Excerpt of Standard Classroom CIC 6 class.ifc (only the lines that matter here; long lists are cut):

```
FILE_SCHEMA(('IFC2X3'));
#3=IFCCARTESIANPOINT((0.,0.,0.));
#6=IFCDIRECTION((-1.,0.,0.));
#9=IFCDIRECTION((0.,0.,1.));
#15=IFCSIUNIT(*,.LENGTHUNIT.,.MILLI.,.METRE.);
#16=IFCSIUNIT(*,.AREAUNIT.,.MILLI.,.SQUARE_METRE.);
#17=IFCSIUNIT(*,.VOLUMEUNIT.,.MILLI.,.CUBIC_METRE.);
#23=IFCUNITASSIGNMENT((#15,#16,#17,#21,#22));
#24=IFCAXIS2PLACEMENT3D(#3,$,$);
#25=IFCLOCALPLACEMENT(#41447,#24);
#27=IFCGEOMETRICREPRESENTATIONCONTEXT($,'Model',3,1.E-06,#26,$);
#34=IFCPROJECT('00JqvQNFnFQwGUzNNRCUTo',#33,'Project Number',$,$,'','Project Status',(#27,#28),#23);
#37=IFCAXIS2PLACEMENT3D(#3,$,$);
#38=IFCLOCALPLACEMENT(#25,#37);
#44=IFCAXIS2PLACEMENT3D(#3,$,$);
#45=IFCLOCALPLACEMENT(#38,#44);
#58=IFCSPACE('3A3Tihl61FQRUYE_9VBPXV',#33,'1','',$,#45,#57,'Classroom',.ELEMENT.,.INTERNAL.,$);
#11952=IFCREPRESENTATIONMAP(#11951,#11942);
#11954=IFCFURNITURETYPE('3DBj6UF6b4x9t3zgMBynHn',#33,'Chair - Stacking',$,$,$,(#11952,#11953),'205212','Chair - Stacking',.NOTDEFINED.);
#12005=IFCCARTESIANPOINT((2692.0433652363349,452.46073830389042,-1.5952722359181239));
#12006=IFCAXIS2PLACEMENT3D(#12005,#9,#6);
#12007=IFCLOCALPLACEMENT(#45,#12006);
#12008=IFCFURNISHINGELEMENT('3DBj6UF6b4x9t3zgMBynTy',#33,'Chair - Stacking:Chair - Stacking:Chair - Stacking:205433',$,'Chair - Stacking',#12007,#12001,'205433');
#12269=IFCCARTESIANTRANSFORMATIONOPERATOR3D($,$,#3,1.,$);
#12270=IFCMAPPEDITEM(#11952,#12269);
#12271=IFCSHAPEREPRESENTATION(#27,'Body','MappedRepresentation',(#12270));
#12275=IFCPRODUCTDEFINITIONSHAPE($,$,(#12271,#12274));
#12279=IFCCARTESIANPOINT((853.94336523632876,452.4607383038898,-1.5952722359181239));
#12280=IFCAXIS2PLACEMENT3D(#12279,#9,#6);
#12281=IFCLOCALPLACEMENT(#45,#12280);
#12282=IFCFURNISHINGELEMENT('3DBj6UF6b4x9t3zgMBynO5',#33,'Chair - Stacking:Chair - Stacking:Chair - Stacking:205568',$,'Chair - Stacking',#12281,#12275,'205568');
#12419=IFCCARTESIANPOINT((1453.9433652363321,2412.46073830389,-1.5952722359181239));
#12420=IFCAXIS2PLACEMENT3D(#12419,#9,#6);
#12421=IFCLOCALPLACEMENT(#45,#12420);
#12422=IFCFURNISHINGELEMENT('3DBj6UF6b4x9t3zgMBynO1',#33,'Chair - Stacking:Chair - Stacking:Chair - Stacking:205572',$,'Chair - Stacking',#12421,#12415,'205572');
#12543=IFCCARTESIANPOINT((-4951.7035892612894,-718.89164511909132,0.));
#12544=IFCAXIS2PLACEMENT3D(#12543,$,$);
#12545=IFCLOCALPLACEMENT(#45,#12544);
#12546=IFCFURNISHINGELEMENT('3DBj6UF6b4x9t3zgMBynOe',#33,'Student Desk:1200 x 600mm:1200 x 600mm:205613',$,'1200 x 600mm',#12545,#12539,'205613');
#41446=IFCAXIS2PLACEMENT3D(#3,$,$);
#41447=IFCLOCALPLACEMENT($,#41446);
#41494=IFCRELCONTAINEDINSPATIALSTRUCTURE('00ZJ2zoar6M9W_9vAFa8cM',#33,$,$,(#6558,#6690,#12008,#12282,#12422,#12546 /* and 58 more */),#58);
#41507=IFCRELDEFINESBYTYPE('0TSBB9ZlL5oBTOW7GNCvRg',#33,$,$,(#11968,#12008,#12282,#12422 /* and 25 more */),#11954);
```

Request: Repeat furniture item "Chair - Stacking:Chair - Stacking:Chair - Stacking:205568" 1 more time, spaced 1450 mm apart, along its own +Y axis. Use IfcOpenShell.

```python
import ifcopenshell
import ifcopenshell.api.geometry
import ifcopenshell.api.root
import ifcopenshell.util.element
import ifcopenshell.util.placement

model = ifcopenshell.open("Standard Classroom CIC 6 class.ifc")


def reuse_history(source, copy):
    """copy_class also copies each property set's owner history, people and application; keep the originals."""
    for rel in copy.IsDefinedBy:
        if rel.is_a("IfcRelDefinesByProperties") and (history := rel.RelatingPropertyDefinition.OwnerHistory):
            rel.RelatingPropertyDefinition.OwnerHistory = source.OwnerHistory
            ifcopenshell.util.element.remove_deep2(model, history)


source = model.by_guid("3DBj6UF6b4x9t3zgMBynO5")
base = ifcopenshell.util.placement.get_local_placement(source.ObjectPlacement)
step = base[:3, 1] * 1450.0

for i in range(1, 2):
    copy = ifcopenshell.api.root.copy_class(model, product=source)
    copy.Representation = ifcopenshell.util.element.copy_deep(
        model, source.Representation, exclude=["IfcGeometricRepresentationContext", "IfcRepresentationMap"]
    )
    copy.Name = "Chair - Stacking:Chair - Stacking:Chair - Stacking"
    copy.Tag = None
    reuse_history(source, copy)
    matrix = base.copy()
    matrix[:3, 3] += i * step
    print("added at", matrix[:3, 3].round(3) + 0.0)
    ifcopenshell.api.geometry.edit_object_placement(model, product=copy, matrix=matrix, is_si=False)

model.write("Standard Classroom CIC 6 class_v2.ifc")
```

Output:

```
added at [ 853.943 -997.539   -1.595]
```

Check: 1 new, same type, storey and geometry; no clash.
